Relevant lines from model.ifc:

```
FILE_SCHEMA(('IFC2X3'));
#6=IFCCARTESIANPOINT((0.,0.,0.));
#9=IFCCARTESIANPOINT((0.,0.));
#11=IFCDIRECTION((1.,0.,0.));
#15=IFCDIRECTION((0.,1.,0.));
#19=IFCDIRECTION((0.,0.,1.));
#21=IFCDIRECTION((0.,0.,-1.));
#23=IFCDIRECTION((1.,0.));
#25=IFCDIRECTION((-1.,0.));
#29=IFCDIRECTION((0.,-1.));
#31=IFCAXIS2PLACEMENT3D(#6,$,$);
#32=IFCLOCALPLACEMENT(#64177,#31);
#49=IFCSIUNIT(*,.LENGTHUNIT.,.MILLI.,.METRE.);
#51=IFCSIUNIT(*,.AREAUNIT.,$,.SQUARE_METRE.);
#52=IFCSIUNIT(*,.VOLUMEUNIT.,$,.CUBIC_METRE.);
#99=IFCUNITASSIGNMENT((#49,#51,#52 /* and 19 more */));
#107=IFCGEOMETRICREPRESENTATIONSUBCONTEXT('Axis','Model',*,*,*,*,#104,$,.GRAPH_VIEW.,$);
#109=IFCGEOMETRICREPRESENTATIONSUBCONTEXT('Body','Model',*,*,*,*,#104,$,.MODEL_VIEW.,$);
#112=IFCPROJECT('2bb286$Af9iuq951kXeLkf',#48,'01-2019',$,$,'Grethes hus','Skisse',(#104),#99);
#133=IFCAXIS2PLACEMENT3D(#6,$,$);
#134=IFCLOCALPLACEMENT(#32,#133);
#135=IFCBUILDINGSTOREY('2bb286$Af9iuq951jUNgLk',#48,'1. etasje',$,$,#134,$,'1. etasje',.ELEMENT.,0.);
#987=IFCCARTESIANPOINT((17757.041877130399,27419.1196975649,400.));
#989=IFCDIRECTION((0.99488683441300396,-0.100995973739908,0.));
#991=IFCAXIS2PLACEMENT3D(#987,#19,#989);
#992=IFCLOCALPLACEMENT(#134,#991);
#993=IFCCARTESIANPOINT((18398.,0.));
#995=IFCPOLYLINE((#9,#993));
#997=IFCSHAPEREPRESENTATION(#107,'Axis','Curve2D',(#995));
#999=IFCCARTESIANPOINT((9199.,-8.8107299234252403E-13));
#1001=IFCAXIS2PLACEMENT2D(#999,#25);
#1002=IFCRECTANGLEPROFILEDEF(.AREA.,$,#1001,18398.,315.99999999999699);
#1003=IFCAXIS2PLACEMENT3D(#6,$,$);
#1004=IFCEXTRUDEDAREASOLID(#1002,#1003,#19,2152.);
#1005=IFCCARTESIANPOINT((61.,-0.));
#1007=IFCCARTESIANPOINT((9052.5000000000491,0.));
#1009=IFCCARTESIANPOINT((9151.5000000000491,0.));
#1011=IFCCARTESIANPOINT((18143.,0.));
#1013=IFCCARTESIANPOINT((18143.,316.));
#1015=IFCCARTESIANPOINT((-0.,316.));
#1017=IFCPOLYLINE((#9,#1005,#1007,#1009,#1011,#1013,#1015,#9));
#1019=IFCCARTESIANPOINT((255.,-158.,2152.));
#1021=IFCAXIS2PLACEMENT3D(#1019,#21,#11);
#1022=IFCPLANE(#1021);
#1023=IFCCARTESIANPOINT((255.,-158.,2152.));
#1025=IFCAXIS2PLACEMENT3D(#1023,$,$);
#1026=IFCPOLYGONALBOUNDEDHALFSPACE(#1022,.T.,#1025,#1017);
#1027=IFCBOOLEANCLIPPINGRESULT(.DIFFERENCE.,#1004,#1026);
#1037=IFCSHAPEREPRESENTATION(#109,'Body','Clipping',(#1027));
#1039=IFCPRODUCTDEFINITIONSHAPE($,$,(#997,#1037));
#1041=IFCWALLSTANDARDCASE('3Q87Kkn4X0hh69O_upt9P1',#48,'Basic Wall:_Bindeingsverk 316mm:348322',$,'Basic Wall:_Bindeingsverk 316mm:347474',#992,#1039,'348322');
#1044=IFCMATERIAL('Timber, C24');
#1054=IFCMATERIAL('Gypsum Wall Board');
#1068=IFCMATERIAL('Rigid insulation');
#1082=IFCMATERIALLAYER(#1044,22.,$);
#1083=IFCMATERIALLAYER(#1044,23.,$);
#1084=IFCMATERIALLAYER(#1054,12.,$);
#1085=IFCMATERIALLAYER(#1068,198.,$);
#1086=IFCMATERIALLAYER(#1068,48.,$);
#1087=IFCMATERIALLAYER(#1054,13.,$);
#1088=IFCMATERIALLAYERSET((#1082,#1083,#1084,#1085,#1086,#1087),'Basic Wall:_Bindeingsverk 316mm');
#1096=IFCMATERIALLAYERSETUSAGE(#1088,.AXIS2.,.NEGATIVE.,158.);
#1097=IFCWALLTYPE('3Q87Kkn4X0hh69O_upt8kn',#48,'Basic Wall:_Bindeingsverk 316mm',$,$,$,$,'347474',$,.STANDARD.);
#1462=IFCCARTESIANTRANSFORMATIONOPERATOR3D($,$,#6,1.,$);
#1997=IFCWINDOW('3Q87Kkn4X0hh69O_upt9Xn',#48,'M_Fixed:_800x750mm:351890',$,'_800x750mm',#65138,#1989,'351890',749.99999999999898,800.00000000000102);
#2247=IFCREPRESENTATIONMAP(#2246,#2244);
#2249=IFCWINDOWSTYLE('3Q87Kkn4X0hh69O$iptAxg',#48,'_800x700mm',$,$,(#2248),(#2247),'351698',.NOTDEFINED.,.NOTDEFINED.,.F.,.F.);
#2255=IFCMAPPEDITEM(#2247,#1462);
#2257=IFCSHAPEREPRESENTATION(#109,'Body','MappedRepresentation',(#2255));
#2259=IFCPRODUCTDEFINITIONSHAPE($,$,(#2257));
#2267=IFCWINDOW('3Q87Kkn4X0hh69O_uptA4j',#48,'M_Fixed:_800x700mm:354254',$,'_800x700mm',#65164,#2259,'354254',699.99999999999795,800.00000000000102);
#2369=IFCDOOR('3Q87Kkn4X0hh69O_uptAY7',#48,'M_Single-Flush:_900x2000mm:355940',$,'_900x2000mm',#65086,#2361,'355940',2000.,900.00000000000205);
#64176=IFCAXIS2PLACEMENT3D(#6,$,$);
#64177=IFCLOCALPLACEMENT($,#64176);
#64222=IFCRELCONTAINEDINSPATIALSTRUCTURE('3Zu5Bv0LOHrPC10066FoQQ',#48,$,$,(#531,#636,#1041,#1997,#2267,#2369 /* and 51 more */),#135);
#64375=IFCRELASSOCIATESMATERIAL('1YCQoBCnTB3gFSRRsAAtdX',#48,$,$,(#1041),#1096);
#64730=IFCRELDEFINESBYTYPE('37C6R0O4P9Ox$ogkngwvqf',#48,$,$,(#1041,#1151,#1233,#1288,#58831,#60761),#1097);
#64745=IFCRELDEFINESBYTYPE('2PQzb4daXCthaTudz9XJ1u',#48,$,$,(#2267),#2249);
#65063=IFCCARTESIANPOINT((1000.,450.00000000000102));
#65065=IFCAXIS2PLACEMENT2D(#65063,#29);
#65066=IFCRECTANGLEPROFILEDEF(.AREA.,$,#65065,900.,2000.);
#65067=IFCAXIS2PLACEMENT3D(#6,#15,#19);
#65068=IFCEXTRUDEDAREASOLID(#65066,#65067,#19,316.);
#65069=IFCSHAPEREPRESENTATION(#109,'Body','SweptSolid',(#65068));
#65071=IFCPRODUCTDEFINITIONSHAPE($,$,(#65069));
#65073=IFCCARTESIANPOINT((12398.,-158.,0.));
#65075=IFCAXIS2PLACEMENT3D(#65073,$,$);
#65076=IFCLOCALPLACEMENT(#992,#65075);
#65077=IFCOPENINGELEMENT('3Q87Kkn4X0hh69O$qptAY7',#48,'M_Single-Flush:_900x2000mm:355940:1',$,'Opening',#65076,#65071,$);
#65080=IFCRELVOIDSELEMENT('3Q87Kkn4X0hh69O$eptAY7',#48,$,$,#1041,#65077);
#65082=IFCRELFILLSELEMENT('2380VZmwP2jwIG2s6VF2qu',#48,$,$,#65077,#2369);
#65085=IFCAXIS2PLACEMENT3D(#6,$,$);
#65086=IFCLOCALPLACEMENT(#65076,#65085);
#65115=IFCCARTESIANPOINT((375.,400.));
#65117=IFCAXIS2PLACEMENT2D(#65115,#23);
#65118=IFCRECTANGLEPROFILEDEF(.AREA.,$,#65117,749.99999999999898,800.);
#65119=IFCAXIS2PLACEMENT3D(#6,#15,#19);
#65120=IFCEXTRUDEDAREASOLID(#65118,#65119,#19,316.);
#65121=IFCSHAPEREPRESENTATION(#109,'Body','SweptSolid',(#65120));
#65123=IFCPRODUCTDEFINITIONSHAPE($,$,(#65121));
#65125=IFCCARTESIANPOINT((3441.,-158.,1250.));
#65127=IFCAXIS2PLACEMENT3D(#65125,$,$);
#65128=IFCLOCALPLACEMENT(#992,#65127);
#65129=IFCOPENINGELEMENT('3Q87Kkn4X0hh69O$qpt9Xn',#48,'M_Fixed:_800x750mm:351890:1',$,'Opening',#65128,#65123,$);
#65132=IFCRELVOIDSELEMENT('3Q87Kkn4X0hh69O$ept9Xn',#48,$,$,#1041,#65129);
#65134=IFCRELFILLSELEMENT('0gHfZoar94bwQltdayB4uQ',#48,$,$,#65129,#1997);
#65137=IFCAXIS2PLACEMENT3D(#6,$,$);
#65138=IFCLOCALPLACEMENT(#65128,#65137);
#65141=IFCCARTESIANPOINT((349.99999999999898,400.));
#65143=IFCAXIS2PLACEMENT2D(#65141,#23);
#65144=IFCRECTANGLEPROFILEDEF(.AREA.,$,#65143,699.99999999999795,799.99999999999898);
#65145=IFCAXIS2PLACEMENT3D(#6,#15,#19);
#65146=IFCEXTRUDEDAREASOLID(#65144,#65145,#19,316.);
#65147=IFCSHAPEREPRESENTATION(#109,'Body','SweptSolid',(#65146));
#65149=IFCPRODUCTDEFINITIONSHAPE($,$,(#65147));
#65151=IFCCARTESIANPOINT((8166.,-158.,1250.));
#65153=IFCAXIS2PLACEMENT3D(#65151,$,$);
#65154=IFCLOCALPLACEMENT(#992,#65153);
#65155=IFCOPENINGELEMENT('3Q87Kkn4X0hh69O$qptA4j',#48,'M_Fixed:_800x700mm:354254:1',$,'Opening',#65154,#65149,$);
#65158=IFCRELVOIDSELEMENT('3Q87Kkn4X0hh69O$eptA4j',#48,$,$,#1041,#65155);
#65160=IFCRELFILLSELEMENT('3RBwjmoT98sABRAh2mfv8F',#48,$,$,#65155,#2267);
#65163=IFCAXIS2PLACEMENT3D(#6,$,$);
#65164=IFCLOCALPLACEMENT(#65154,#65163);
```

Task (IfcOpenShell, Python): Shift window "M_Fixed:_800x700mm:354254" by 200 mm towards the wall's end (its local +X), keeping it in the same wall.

```python
import ifcopenshell
import ifcopenshell.api.geometry
import ifcopenshell.util.placement
import ifcopenshell.util.unit

model = ifcopenshell.open("model.ifc")
unit_scale = ifcopenshell.util.unit.calculate_unit_scale(model)

window = model.by_guid("3Q87Kkn4X0hh69O_uptA4j")
opening = window.FillsVoids[0].RelatingOpeningElement
wall = opening.VoidsElements[0].RelatingBuildingElement

wall_matrix = ifcopenshell.util.placement.get_local_placement(wall.ObjectPlacement)
shift = wall_matrix[:3, 0] * 0.2 / unit_scale
before = ifcopenshell.util.placement.get_local_placement(window.ObjectPlacement)[:3, 3].copy()

# The window is placed relative to its opening, so it follows when the opening moves.
matrix = ifcopenshell.util.placement.get_local_placement(opening.ObjectPlacement)
matrix[:3, 3] += shift
ifcopenshell.api.geometry.edit_object_placement(
    model, product=opening, matrix=matrix, is_si=False, should_transform_children=True
)

after = ifcopenshell.util.placement.get_local_placement(window.ObjectPlacement)[:3, 3]
print("window moved by", (after - before).round(3) + 0.0)

model.write("model_edited.ifc")
```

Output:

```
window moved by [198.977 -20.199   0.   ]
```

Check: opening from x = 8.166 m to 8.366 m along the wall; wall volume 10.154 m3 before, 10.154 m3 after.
